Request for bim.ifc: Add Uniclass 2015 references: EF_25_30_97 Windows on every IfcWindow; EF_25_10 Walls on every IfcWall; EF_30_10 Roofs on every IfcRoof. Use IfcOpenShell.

First a look at what the model holds.

```python
import ifcopenshell

model = ifcopenshell.open("bim.ifc")
print(model.schema)
print("classifications:", [c.Name for c in model.by_type("IfcClassification")])
for ifc_class in ("IfcDoor", "IfcRoof", "IfcStair", "IfcWall", "IfcWindow"):
    print(ifc_class, len(model.by_type(ifc_class)))
```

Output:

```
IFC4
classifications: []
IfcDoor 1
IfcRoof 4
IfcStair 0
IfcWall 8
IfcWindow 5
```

```python
import ifcopenshell
import ifcopenshell.api.classification

model = ifcopenshell.open("bim.ifc")

system = ifcopenshell.api.classification.add_classification(model, classification="Uniclass 2015")

codes = {
    "IfcWindow": ("EF_25_30_97", "Windows"),
    "IfcWall": ("EF_25_10", "Walls"),
    "IfcRoof": ("EF_30_10", "Roofs"),
}
for ifc_class, (code, name) in codes.items():
    products = model.by_type(ifc_class)
    ifcopenshell.api.classification.add_reference(
        model, products=products, classification=system, identification=code, name=name
    )
    print(code, len(products))

model.write("bim_edited.ifc")
```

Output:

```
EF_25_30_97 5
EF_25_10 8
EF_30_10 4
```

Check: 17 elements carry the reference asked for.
